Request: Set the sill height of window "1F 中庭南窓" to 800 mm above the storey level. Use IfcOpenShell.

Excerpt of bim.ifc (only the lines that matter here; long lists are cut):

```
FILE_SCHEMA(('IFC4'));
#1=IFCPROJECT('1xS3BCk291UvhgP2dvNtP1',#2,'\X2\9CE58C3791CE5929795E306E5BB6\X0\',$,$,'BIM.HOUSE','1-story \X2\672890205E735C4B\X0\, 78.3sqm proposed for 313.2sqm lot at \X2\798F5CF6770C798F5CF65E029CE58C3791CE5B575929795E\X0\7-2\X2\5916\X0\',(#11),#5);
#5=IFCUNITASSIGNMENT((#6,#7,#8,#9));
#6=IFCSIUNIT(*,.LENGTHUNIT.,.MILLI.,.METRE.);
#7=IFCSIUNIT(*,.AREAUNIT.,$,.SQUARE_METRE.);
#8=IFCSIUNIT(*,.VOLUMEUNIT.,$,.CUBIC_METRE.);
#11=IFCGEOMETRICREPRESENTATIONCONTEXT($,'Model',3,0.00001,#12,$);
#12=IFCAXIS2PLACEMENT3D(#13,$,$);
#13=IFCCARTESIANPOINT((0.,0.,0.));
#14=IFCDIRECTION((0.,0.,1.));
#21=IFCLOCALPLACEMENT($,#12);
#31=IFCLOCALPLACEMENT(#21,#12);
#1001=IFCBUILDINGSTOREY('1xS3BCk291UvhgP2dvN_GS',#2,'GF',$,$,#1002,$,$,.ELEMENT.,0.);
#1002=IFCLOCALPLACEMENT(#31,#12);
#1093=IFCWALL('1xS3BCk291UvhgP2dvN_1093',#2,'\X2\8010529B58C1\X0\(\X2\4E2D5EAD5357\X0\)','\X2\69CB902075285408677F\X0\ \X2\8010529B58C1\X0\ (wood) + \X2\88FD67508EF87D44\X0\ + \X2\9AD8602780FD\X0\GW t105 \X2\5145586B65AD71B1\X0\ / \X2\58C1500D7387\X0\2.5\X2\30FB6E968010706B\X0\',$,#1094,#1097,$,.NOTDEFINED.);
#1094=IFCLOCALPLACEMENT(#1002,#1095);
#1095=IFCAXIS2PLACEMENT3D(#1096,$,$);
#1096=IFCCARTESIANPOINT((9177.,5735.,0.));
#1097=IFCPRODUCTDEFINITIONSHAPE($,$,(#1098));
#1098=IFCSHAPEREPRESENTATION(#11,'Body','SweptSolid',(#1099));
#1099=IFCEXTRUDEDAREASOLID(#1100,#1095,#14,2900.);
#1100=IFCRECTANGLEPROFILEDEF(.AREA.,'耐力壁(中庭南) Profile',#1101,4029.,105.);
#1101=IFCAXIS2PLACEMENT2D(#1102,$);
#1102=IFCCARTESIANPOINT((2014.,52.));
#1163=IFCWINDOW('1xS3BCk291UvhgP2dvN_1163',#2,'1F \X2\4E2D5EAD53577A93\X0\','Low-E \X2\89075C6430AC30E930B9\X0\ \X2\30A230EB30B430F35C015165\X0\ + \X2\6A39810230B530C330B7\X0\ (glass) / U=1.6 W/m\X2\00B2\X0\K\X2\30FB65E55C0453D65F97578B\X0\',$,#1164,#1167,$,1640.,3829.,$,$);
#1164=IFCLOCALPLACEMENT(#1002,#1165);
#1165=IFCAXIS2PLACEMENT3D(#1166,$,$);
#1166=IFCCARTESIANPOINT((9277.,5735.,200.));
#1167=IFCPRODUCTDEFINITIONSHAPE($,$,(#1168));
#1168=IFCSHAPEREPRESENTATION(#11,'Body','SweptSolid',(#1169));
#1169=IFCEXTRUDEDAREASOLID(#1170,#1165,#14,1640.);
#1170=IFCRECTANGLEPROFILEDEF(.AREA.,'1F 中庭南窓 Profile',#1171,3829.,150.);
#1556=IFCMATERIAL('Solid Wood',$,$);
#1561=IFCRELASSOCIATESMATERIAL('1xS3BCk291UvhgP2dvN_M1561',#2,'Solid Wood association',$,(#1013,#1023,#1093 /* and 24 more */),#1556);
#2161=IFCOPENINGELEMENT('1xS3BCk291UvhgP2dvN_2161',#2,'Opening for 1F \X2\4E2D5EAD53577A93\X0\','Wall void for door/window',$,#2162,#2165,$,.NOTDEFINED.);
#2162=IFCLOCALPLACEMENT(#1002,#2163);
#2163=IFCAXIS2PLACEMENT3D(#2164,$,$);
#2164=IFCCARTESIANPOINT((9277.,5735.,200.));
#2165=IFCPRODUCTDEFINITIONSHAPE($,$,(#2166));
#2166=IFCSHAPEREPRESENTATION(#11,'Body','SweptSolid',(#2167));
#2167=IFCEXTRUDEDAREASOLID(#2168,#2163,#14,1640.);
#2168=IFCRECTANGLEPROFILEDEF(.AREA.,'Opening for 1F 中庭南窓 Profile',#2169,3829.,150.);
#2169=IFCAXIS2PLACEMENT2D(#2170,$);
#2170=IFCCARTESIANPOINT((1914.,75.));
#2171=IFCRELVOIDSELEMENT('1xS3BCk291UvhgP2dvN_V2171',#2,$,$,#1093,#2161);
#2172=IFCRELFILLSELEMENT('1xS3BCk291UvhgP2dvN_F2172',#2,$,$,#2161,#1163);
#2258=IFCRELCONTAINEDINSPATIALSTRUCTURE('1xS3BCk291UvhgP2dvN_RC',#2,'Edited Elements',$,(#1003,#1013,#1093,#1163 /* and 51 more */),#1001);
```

```python
import numpy as np
import ifcopenshell
import ifcopenshell.api.geometry
import ifcopenshell.geom
import ifcopenshell.util.element
import ifcopenshell.util.placement
import ifcopenshell.util.shape
import ifcopenshell.util.unit

model = ifcopenshell.open("bim.ifc")
unit_scale = ifcopenshell.util.unit.calculate_unit_scale(model)

window = model.by_guid("1xS3BCk291UvhgP2dvN_1163")
opening = window.FillsVoids[0].RelatingOpeningElement
storey = ifcopenshell.util.element.get_container(window, ifc_class="IfcBuildingStorey")
level = ifcopenshell.util.placement.get_local_placement(storey.ObjectPlacement)[2, 3]

# The opening's origin need not be at the sill, so measure its lowest point.
shape = ifcopenshell.geom.create_shape(ifcopenshell.geom.settings(), opening)
bottom = ifcopenshell.util.shape.get_shape_bottom_elevation(shape, shape.geometry) / unit_scale
dz = level + 0.8 / unit_scale - bottom

shift = np.array([0.0, 0.0, dz])
# The window is not placed relative to its opening, so move both.
for product in (opening, window):
    matrix = ifcopenshell.util.placement.get_local_placement(product.ObjectPlacement)
    matrix[:3, 3] += shift
    ifcopenshell.api.geometry.edit_object_placement(model, product=product, matrix=matrix, is_si=False)

print(f"moved by {dz * unit_scale:+.3f} m")

model.write("bim_rev.ifc")
```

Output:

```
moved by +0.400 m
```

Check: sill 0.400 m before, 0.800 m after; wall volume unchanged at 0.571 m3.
